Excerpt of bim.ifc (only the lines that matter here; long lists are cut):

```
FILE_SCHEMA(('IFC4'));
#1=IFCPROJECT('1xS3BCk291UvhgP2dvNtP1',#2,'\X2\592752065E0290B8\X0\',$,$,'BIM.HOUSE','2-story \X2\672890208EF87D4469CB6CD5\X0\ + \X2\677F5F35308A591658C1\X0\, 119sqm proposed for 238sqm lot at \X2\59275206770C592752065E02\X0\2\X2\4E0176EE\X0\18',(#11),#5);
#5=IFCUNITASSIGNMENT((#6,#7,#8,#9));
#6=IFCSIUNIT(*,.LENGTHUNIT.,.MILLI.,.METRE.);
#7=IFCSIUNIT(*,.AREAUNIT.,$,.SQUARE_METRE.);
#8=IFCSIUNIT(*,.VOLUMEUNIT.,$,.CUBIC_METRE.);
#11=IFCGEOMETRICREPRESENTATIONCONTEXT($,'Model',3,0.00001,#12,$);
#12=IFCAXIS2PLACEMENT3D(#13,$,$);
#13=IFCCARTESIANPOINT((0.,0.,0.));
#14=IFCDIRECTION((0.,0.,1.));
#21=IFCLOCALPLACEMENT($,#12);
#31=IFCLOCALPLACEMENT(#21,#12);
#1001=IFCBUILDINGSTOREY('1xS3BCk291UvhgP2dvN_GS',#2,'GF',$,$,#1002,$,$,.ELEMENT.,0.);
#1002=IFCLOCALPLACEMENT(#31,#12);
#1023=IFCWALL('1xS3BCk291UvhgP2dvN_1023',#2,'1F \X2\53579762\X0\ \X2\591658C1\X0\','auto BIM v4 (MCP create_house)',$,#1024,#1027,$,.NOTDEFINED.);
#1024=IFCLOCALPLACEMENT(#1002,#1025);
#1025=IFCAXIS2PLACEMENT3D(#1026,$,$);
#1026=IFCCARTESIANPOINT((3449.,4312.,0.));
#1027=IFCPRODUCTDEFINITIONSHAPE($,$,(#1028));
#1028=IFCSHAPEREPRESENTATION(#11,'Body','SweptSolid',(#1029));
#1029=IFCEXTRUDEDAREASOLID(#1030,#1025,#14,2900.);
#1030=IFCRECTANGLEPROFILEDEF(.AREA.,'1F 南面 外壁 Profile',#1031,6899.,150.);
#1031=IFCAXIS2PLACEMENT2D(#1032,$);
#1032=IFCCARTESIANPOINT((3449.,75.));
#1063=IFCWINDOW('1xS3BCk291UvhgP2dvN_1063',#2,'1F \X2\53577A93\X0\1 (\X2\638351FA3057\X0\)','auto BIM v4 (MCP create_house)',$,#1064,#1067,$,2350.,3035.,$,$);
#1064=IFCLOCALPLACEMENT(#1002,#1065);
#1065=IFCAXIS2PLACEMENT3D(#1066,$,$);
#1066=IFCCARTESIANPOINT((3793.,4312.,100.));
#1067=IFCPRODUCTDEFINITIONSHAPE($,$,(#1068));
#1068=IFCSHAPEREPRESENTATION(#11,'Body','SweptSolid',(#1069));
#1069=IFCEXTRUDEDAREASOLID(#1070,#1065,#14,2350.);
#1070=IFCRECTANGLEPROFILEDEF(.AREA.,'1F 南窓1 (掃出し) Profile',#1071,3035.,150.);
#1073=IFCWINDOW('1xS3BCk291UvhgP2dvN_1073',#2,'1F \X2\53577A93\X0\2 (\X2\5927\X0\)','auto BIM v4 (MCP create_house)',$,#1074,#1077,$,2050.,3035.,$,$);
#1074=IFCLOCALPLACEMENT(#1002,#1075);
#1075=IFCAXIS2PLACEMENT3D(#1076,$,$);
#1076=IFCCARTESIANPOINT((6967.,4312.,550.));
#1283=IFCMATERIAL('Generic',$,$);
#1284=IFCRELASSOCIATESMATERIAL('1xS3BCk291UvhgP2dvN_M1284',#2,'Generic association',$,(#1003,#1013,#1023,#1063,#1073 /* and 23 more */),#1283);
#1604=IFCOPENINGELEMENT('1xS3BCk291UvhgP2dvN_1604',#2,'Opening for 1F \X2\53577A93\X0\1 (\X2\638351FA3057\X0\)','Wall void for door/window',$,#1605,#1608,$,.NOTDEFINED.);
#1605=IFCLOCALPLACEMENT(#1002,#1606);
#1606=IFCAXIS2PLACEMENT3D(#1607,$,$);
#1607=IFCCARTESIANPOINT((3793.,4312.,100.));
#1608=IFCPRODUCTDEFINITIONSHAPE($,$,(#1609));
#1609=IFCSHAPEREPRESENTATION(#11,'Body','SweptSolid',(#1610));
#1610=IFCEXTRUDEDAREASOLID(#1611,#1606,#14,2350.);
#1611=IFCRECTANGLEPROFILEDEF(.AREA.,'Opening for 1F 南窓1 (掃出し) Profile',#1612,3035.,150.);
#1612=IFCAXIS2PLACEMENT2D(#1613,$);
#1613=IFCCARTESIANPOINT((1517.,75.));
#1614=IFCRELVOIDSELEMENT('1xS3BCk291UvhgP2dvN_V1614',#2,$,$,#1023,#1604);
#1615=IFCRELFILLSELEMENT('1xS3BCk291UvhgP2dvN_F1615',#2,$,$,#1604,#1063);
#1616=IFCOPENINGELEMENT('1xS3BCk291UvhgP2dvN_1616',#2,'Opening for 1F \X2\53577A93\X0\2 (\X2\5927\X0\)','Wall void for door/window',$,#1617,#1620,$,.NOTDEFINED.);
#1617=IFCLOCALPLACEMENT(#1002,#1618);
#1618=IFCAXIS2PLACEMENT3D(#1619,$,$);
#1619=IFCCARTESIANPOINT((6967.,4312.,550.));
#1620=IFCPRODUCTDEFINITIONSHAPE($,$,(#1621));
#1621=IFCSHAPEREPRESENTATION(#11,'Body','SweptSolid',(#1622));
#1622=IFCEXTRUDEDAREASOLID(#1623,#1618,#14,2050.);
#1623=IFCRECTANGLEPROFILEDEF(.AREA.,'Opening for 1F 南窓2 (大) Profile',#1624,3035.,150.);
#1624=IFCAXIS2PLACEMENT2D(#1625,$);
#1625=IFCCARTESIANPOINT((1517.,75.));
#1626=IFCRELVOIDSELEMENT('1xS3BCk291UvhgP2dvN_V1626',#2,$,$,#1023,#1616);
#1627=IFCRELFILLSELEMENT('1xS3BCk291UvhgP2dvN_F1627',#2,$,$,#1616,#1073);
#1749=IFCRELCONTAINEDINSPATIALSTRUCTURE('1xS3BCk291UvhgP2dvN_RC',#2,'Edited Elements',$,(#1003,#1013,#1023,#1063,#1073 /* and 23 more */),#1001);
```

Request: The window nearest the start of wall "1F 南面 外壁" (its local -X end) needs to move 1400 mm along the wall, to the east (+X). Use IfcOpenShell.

```python
import ifcopenshell
import ifcopenshell.api.geometry
import ifcopenshell.util.placement

model = ifcopenshell.open("bim.ifc")

window = model.by_id(1063)
opening = window.FillsVoids[0].RelatingOpeningElement
wall = opening.VoidsElements[0].RelatingBuildingElement

wall_matrix = ifcopenshell.util.placement.get_local_placement(wall.ObjectPlacement)
shift = wall_matrix[:3, 0] * 1400.0
before = ifcopenshell.util.placement.get_local_placement(window.ObjectPlacement)[:3, 3].copy()

# The window is not placed relative to its opening, so move both.
for product in (opening, window):
    matrix = ifcopenshell.util.placement.get_local_placement(product.ObjectPlacement)
    matrix[:3, 3] += shift
    ifcopenshell.api.geometry.edit_object_placement(model, product=product, matrix=matrix, is_si=False)

after = ifcopenshell.util.placement.get_local_placement(window.ObjectPlacement)[:3, 3]
print("window moved by", (after - before).round(3) + 0.0)

model.write("bim_edited.ifc")
```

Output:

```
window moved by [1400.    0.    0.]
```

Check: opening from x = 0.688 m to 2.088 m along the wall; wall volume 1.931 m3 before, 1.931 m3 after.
